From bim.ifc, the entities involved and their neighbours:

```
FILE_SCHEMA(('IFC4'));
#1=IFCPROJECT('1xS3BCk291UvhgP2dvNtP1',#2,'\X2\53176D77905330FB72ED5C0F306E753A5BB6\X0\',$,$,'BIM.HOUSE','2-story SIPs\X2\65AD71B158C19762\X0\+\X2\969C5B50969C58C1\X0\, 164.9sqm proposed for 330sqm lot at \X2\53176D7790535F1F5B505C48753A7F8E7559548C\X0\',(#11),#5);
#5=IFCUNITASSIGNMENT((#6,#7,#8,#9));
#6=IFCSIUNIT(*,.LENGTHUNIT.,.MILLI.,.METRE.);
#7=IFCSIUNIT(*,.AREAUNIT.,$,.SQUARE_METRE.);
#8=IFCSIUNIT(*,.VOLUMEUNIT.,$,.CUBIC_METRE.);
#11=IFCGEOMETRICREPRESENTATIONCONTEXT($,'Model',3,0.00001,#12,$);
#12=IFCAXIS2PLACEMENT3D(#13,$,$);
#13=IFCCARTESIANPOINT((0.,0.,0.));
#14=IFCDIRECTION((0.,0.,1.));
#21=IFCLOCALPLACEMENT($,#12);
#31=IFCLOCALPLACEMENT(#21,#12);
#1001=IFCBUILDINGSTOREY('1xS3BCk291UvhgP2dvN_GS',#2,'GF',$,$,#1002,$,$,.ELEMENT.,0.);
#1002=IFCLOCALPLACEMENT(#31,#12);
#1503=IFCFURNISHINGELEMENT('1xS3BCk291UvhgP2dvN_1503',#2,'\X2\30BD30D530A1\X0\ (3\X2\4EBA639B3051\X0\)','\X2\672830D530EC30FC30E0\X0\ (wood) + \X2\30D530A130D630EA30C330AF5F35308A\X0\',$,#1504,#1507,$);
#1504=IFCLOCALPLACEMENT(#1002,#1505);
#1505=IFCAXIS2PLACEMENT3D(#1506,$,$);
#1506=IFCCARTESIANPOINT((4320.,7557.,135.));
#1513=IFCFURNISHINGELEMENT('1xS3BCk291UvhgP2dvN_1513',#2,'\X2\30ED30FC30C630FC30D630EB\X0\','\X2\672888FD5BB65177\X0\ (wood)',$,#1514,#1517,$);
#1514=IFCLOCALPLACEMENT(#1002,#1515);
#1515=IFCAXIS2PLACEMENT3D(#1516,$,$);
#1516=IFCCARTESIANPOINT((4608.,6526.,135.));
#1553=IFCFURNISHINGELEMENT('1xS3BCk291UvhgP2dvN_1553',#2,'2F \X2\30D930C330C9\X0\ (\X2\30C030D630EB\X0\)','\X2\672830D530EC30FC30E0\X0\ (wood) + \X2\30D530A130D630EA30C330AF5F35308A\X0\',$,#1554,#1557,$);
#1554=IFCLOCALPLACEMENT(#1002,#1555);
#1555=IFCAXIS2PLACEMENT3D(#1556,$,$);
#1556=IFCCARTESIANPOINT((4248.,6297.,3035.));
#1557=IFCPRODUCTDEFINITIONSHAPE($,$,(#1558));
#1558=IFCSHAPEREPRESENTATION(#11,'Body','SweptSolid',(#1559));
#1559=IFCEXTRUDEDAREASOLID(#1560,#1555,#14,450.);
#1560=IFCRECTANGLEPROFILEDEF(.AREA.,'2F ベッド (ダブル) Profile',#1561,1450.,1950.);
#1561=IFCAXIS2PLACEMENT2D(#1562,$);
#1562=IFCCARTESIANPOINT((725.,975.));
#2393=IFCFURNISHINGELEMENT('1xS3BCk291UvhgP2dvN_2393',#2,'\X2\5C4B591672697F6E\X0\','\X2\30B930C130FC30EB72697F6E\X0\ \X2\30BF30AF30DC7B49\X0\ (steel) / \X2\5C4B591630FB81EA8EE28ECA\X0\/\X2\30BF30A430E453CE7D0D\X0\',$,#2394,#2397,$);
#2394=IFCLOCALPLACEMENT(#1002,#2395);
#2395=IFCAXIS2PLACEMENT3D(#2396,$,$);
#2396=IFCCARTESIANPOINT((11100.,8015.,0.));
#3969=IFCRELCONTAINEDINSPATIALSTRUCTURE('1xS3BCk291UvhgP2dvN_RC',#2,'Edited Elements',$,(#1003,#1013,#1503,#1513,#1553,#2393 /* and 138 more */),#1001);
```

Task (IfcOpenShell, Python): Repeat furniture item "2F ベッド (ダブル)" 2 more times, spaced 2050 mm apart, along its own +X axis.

```python
import ifcopenshell
import ifcopenshell.api.geometry
import ifcopenshell.api.root
import ifcopenshell.util.element
import ifcopenshell.util.placement
import ifcopenshell.util.unit

model = ifcopenshell.open("bim.ifc")
unit_scale = ifcopenshell.util.unit.calculate_unit_scale(model)


def reuse_history(source, copy):
    """copy_class also copies each property set's owner history, people and application; keep the originals."""
    for rel in copy.IsDefinedBy:
        if rel.is_a("IfcRelDefinesByProperties") and (history := rel.RelatingPropertyDefinition.OwnerHistory):
            rel.RelatingPropertyDefinition.OwnerHistory = source.OwnerHistory
            ifcopenshell.util.element.remove_deep2(model, history)


source = model.by_guid("1xS3BCk291UvhgP2dvN_1553")
base = ifcopenshell.util.placement.get_local_placement(source.ObjectPlacement)
step = base[:3, 0] * 2.05 / unit_scale

for i in range(1, 3):
    copy = ifcopenshell.api.root.copy_class(model, product=source)
    copy.Representation = ifcopenshell.util.element.copy_deep(
        model, source.Representation, exclude=["IfcGeometricRepresentationContext", "IfcRepresentationMap"]
    )
    reuse_history(source, copy)
    matrix = base.copy()
    matrix[:3, 3] += i * step
    print("added at", matrix[:3, 3].round(3) + 0.0)
    ifcopenshell.api.geometry.edit_object_placement(model, product=copy, matrix=matrix, is_si=False)

model.write("bim_edited.ifc")
```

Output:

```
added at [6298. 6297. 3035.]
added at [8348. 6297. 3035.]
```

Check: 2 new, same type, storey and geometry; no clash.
